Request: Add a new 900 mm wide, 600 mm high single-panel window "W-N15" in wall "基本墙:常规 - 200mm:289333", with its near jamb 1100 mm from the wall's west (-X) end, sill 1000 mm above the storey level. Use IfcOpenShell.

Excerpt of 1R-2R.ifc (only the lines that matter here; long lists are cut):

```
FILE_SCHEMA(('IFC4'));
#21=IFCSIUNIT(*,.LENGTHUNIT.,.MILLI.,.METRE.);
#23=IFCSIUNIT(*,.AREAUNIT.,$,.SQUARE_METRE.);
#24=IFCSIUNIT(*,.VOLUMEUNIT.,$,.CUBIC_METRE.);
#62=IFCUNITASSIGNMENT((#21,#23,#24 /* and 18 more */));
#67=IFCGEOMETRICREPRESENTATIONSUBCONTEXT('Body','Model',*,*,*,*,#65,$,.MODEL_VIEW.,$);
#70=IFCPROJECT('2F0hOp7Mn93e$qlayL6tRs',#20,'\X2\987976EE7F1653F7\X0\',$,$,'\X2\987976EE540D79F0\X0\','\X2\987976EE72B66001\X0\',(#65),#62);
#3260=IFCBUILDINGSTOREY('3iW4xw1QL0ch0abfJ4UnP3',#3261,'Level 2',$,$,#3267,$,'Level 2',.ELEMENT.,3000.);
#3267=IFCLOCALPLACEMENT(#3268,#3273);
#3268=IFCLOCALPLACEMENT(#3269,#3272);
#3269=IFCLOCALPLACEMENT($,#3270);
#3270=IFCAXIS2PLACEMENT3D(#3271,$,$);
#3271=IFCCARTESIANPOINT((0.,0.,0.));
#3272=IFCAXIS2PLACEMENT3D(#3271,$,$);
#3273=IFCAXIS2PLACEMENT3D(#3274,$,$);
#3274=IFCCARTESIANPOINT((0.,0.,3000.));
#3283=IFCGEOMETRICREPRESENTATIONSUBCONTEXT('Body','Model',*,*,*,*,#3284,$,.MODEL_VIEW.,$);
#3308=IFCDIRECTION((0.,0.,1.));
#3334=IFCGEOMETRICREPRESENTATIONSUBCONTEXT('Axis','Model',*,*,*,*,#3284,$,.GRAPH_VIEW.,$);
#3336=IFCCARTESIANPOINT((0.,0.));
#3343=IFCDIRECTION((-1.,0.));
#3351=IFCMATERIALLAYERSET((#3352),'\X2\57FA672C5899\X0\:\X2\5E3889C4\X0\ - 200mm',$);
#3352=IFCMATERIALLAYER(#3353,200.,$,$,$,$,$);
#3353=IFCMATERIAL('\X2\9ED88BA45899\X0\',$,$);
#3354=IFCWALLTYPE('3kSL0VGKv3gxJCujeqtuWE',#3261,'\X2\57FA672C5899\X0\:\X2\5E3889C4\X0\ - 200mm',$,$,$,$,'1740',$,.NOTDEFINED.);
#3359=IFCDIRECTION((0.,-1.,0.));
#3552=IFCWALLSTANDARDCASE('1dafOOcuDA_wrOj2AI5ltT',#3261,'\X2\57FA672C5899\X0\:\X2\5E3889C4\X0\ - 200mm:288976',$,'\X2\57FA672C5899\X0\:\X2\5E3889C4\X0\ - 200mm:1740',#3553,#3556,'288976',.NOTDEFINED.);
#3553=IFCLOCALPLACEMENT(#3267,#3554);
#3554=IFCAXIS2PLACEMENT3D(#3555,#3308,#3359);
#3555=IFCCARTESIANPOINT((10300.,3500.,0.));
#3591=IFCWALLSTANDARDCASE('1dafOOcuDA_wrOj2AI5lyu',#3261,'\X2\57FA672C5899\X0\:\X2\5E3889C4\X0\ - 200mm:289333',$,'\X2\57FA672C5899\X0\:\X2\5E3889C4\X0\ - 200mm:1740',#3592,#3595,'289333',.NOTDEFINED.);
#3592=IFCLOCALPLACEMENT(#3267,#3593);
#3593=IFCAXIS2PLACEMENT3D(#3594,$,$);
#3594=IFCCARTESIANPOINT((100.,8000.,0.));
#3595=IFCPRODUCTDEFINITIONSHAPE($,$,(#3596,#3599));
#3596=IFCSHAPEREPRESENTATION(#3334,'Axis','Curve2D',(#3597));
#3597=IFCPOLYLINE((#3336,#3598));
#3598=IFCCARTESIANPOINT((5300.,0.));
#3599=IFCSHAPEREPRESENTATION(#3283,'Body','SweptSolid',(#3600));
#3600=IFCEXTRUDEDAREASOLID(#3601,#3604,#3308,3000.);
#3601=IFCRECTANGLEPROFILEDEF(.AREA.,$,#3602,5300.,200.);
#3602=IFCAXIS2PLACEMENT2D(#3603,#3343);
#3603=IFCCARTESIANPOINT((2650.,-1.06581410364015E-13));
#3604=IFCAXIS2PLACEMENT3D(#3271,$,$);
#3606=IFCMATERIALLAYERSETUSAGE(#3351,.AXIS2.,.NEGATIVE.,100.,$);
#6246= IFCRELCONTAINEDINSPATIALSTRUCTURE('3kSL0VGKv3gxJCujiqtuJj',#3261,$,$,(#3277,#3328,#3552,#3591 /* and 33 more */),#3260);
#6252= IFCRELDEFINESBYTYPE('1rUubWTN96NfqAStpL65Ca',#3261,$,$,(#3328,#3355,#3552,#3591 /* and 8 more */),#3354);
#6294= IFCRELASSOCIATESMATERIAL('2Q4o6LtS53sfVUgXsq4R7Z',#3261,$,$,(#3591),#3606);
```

```python
import numpy as np
import ifcopenshell
import ifcopenshell.api.feature
import ifcopenshell.api.geometry
import ifcopenshell.api.root
import ifcopenshell.api.spatial
import ifcopenshell.geom
import ifcopenshell.util.element
import ifcopenshell.util.placement
import ifcopenshell.util.representation
import ifcopenshell.util.shape
import ifcopenshell.util.unit

model = ifcopenshell.open("1R-2R.ifc")
unit_scale = ifcopenshell.util.unit.calculate_unit_scale(model)
settings = ifcopenshell.geom.settings()


def volume(element):
    """Net volume in cubic metres, openings subtracted."""
    shape = ifcopenshell.geom.create_shape(settings, element)
    return ifcopenshell.util.shape.get_volume(shape.geometry)


wall = model.by_guid("1dafOOcuDA_wrOj2AI5lyu")
storey = ifcopenshell.util.element.get_container(wall, ifc_class="IfcBuildingStorey")
context = ifcopenshell.util.representation.get_context(model, "Model", "Body", "MODEL_VIEW")
before = volume(wall)

width, height, from_end, sill = 0.9, 0.6, 1.1, 1  # metres

# The wall runs along its own X axis, and the end named is its -X end.
wall_shape = ifcopenshell.geom.create_shape(settings, wall)
x, y, z = ifcopenshell.util.shape.get_vertices(wall_shape.geometry).T
start = x.min() + from_end
face, thickness = float(y.min()), float(y.max() - y.min())
wall_matrix = ifcopenshell.util.placement.get_local_placement(wall.ObjectPlacement)
level = ifcopenshell.util.placement.get_local_placement(storey.ObjectPlacement)[2, 3]


def in_wall(x, y):
    """Placement at x, y metres in the wall's axes, at sill height."""
    matrix = wall_matrix.copy()
    matrix[:, 3] = wall_matrix @ np.array([x / unit_scale, y / unit_scale, 0.0, 1.0])
    matrix[2, 3] = level + sill / unit_scale
    return matrix


# Opening: a box that overshoots both wall faces by 50 mm.
opening = ifcopenshell.api.root.create_entity(model, ifc_class="IfcOpeningElement", predefined_type="OPENING")
box = ifcopenshell.api.geometry.add_wall_representation(
    model, context=context, length=width, height=height, thickness=thickness + 0.1
)
ifcopenshell.api.geometry.assign_representation(model, product=opening, representation=box)
ifcopenshell.api.geometry.edit_object_placement(model, product=opening, matrix=in_wall(start, face - 0.05), is_si=False)
ifcopenshell.api.feature.add_feature(model, feature=opening, element=wall)

window = ifcopenshell.api.root.create_entity(model, ifc_class="IfcWindow", name="W-N15", predefined_type="WINDOW")
window.OverallWidth, window.OverallHeight = width / unit_scale, height / unit_scale
window.PartitioningType = "SINGLE_PANEL"
body = ifcopenshell.api.geometry.add_window_representation(
    model,
    context=context,
    overall_width=window.OverallWidth,
    overall_height=window.OverallHeight,
    partition_type="SINGLE_PANEL",
)
ifcopenshell.api.geometry.assign_representation(model, product=window, representation=body)
ifcopenshell.api.spatial.assign_container(model, products=[window], relating_structure=storey)
ifcopenshell.api.feature.add_filling(model, opening=opening, element=window)

# Centre the window in the wall's thickness.
ifcopenshell.api.geometry.edit_object_placement(model, product=window, matrix=in_wall(start, face), is_si=False)
window_shape = ifcopenshell.geom.create_shape(settings, window)
depth = ifcopenshell.util.shape.get_vertices(window_shape.geometry)[:, 1]
offset = face + thickness / 2 - (depth.min() + depth.max()) / 2
ifcopenshell.api.geometry.edit_object_placement(model, product=window, matrix=in_wall(start, offset), is_si=False)

after = volume(wall)

print(f"wall volume {before:.3f} -> {after:.3f} m3")

model.write("1R-2R_rev.ifc")
```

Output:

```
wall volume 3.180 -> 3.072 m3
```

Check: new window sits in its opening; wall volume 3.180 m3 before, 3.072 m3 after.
